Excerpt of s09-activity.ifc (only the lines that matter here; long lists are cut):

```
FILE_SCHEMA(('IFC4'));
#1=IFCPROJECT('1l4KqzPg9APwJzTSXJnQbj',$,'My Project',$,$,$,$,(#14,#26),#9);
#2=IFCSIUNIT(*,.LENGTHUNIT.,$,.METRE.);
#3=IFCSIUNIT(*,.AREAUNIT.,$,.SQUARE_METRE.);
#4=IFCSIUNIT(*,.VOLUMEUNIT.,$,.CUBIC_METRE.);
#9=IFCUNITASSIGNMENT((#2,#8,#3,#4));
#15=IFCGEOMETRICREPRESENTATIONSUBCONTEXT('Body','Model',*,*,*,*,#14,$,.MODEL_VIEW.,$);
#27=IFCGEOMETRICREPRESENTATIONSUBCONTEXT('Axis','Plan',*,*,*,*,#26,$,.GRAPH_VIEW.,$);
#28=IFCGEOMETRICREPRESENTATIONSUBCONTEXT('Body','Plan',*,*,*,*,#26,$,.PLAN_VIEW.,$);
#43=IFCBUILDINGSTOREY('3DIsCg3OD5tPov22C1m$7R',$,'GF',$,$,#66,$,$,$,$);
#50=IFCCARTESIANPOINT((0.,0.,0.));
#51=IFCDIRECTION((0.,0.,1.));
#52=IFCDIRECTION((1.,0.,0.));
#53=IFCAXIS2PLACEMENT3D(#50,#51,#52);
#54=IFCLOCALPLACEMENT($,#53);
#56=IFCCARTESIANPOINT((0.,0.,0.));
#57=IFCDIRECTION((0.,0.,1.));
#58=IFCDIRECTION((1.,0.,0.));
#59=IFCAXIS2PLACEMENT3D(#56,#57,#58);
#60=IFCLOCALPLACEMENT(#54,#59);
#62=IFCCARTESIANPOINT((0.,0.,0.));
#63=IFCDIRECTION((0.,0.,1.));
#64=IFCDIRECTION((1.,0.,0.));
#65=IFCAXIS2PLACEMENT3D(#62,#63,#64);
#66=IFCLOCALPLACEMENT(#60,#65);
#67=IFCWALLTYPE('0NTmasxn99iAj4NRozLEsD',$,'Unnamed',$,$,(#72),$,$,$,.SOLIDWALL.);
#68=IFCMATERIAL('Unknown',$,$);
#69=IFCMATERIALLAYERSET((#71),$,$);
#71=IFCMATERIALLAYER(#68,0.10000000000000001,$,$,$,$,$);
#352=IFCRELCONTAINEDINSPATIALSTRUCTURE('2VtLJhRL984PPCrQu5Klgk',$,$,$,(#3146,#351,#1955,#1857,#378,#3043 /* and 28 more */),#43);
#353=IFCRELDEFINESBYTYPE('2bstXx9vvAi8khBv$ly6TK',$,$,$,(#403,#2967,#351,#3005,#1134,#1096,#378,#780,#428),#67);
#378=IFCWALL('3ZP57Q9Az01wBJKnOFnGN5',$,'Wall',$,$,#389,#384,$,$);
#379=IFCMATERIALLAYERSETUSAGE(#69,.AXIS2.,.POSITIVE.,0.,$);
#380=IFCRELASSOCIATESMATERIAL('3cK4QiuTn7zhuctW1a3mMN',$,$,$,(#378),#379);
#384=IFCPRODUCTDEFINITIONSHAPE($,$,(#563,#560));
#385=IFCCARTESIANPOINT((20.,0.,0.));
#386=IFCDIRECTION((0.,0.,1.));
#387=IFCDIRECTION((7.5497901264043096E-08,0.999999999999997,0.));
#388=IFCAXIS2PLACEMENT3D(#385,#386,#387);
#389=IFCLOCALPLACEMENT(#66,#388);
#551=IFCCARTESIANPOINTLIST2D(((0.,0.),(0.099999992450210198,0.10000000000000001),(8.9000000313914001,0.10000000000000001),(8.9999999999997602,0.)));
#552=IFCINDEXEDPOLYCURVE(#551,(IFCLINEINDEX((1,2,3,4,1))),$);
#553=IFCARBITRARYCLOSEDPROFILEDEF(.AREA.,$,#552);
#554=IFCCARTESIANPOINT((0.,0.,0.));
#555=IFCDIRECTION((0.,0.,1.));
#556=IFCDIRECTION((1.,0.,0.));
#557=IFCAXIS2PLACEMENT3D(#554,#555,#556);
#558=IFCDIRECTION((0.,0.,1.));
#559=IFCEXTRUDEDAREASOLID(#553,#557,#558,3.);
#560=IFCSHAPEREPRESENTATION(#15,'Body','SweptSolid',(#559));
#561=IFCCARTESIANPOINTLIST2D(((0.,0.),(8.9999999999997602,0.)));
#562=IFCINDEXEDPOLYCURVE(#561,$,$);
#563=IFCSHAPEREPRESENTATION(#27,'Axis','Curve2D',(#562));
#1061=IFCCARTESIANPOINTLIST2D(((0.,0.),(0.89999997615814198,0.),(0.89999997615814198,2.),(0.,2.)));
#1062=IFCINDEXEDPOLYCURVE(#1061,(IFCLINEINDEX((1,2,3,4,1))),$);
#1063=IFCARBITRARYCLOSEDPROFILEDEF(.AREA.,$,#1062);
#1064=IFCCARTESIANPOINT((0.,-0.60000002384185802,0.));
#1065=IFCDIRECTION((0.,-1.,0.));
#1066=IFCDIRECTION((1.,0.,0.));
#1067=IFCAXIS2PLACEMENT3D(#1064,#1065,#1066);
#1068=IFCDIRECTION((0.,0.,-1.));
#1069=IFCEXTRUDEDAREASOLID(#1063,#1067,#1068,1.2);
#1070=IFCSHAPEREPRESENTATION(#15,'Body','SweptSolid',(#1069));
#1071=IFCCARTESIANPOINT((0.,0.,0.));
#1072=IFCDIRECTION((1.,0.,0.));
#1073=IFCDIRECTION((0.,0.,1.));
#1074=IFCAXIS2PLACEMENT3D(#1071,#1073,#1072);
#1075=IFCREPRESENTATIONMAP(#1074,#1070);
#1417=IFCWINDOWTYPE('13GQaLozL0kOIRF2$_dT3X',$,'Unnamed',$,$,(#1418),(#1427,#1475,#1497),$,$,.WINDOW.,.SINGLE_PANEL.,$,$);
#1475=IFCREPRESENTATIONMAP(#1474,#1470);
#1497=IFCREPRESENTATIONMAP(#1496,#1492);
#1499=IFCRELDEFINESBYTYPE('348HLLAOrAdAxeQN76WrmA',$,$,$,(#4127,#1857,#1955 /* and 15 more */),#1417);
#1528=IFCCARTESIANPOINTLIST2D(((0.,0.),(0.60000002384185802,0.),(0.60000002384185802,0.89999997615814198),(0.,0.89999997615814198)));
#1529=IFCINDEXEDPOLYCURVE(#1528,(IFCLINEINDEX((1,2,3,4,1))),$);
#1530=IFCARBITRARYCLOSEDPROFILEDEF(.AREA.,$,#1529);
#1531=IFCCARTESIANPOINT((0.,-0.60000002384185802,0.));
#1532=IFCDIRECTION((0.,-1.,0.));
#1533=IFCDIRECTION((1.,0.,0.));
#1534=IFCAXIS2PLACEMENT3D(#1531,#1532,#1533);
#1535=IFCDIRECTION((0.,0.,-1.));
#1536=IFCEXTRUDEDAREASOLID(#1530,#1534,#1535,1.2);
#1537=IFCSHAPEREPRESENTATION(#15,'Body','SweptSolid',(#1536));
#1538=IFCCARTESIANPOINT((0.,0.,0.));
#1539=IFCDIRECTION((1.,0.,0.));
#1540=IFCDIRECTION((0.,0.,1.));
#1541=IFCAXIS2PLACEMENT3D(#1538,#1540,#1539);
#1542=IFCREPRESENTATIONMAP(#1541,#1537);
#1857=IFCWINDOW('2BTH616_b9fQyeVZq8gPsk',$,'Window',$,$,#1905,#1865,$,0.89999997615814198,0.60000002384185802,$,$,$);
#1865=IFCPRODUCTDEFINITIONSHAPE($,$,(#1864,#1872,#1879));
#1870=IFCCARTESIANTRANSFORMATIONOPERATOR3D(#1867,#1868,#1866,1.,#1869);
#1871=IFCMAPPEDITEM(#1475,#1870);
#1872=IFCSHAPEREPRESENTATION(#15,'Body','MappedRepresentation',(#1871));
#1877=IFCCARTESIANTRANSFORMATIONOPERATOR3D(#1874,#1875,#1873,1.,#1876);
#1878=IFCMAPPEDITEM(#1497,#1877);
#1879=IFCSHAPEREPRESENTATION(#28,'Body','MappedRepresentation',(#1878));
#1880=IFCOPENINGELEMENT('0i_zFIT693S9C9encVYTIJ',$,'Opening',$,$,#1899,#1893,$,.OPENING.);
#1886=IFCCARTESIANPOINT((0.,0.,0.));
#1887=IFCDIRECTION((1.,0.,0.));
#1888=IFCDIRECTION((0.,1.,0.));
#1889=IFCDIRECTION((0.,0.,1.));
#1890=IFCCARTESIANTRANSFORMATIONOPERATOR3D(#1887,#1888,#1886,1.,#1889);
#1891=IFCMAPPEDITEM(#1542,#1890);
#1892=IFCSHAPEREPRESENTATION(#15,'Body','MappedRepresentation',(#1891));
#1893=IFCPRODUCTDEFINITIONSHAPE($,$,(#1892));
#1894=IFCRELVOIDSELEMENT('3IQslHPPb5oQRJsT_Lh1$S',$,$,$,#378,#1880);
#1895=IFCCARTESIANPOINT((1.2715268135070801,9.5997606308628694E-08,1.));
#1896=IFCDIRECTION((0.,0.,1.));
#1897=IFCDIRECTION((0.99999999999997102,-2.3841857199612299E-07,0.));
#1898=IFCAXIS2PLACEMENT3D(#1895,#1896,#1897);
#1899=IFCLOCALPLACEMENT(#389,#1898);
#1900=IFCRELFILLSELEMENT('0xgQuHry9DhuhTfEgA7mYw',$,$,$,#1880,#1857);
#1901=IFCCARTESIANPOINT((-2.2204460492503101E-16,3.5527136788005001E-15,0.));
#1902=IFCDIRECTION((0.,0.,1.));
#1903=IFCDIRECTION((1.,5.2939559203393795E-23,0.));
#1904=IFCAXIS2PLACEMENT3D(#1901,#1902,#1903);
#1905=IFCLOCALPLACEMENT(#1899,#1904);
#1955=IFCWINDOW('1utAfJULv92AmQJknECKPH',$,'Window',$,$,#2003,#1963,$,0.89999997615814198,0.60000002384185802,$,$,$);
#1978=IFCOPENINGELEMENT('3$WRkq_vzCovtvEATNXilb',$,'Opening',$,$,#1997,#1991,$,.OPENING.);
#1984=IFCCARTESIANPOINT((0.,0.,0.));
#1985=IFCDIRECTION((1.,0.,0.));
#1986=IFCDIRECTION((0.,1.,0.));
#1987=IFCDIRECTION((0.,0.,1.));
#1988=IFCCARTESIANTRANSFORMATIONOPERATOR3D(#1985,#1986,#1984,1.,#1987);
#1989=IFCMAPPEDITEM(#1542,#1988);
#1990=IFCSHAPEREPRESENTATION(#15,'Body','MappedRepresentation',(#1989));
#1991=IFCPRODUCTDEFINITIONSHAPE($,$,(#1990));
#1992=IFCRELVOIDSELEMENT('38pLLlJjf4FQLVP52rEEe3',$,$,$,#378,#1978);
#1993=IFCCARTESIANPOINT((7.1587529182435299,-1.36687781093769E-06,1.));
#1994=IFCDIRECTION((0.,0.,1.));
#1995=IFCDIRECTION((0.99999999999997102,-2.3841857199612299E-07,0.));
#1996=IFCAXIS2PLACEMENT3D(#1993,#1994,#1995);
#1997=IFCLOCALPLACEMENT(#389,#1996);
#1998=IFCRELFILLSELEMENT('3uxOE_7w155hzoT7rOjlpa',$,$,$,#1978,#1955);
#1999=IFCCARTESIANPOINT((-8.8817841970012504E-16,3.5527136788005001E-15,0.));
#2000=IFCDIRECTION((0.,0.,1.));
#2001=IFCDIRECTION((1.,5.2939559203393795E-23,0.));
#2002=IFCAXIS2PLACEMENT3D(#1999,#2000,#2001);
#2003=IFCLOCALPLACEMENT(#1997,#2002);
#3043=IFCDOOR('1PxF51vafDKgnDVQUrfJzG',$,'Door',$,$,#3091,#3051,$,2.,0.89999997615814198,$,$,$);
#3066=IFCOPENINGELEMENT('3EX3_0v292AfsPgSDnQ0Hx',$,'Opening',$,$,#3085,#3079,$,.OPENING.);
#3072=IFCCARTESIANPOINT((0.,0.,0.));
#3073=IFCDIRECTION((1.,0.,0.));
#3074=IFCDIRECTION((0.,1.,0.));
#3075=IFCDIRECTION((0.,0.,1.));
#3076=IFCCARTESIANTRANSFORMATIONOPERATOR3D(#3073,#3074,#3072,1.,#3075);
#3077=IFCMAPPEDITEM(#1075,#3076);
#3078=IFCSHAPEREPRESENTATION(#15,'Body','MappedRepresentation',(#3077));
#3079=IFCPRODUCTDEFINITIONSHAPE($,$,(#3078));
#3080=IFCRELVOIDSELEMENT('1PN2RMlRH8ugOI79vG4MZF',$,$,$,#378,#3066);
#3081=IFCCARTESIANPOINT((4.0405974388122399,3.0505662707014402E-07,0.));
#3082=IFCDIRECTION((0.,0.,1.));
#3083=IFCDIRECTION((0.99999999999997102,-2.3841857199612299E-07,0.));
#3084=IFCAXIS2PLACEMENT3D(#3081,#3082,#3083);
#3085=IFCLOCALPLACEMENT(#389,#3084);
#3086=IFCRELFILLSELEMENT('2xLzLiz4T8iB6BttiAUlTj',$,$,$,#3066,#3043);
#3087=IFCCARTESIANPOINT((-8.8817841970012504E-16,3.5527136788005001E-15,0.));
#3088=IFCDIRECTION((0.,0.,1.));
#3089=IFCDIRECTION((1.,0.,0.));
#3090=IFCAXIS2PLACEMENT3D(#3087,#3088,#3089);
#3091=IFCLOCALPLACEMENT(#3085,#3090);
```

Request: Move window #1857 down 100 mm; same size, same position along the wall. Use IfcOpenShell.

```python
import numpy as np
import ifcopenshell
import ifcopenshell.api.geometry
import ifcopenshell.util.placement
import ifcopenshell.util.unit

model = ifcopenshell.open("s09-activity.ifc")
unit_scale = ifcopenshell.util.unit.calculate_unit_scale(model)

window = model.by_guid("2BTH616_b9fQyeVZq8gPsk")
opening = window.FillsVoids[0].RelatingOpeningElement
dz = -0.1 / unit_scale

shift = np.array([0.0, 0.0, dz])
# The window is placed relative to its opening, so it follows when the opening moves.
matrix = ifcopenshell.util.placement.get_local_placement(opening.ObjectPlacement)
matrix[:3, 3] += shift
ifcopenshell.api.geometry.edit_object_placement(
    model, product=opening, matrix=matrix, is_si=False, should_transform_children=True
)

print(f"moved by {dz * unit_scale:+.3f} m")

model.write("s09-activity_updated.ifc")
```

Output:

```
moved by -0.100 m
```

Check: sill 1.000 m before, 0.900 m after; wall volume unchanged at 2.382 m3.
